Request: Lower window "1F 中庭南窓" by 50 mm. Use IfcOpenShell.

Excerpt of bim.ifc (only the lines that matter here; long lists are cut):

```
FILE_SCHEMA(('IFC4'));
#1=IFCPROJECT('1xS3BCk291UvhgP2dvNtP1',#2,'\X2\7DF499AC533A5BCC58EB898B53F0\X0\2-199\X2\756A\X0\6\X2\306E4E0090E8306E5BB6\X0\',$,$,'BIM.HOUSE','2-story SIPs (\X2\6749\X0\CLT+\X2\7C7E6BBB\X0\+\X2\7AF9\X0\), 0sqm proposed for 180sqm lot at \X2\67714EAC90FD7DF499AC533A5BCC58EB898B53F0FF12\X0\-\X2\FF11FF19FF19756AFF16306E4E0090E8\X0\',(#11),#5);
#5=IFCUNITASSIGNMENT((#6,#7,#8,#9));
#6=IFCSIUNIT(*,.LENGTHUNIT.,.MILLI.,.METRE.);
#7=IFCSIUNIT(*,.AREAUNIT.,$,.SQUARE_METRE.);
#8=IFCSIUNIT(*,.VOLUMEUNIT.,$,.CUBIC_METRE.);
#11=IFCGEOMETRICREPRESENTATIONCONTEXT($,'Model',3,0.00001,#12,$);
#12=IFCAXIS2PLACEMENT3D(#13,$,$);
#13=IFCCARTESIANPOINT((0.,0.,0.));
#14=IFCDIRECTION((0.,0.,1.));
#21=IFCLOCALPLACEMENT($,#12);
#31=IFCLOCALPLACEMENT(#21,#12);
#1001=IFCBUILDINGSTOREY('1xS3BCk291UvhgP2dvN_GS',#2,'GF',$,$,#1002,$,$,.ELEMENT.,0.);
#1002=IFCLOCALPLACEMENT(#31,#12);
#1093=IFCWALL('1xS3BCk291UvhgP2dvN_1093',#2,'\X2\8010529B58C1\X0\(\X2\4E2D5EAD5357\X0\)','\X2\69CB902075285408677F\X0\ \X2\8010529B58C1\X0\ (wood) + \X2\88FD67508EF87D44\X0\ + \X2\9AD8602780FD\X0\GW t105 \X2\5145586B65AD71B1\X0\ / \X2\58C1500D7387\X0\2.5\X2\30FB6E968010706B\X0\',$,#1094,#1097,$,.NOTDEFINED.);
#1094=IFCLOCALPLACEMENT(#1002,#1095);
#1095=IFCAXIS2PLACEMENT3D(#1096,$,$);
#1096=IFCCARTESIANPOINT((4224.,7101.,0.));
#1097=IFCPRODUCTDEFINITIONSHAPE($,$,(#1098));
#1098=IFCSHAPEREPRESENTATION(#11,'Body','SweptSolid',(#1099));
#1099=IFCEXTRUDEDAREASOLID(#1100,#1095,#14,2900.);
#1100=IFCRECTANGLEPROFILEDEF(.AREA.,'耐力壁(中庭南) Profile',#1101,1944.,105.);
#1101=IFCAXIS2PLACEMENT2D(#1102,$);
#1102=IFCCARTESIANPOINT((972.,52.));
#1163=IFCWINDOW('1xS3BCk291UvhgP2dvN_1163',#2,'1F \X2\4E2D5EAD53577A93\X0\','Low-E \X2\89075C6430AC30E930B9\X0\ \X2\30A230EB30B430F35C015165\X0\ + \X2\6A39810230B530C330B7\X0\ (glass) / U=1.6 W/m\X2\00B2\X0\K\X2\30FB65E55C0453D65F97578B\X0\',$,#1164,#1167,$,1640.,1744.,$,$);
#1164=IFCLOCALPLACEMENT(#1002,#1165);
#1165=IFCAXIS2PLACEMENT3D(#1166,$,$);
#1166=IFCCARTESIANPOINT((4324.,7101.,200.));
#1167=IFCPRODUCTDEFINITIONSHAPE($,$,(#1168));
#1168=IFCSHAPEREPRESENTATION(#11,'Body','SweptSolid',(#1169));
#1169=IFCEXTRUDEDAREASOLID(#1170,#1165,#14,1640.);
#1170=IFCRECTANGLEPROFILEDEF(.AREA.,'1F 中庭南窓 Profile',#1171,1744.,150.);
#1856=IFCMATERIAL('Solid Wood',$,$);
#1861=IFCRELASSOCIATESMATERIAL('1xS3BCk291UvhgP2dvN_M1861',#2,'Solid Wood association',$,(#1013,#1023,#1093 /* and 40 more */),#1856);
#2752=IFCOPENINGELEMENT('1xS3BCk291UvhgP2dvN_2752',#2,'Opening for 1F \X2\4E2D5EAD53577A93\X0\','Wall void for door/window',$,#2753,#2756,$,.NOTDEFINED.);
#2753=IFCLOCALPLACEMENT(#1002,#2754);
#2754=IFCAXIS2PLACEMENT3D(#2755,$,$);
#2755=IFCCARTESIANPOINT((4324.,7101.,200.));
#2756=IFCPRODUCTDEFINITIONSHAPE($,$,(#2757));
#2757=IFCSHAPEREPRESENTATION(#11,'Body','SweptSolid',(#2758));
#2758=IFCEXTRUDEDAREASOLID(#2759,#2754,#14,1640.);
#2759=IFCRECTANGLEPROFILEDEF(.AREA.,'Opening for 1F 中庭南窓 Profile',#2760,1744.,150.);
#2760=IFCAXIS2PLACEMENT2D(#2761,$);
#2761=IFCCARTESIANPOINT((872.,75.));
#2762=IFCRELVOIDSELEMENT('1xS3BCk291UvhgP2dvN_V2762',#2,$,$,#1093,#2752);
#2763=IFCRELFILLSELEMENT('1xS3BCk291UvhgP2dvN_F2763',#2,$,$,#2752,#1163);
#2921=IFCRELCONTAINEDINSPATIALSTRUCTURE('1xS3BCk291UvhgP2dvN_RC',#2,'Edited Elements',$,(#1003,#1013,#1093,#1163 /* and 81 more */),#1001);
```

```python
import numpy as np
import ifcopenshell
import ifcopenshell.api.geometry
import ifcopenshell.util.placement
import ifcopenshell.util.unit

model = ifcopenshell.open("bim.ifc")
unit_scale = ifcopenshell.util.unit.calculate_unit_scale(model)

window = model.by_guid("1xS3BCk291UvhgP2dvN_1163")
opening = window.FillsVoids[0].RelatingOpeningElement
dz = -0.05 / unit_scale

shift = np.array([0.0, 0.0, dz])
# The window is not placed relative to its opening, so move both.
for product in (opening, window):
    matrix = ifcopenshell.util.placement.get_local_placement(product.ObjectPlacement)
    matrix[:3, 3] += shift
    ifcopenshell.api.geometry.edit_object_placement(model, product=product, matrix=matrix, is_si=False)

print(f"moved by {dz * unit_scale:+.3f} m")

model.write("bim_updated.ifc")
```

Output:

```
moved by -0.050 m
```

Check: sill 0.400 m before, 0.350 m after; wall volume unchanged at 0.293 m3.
